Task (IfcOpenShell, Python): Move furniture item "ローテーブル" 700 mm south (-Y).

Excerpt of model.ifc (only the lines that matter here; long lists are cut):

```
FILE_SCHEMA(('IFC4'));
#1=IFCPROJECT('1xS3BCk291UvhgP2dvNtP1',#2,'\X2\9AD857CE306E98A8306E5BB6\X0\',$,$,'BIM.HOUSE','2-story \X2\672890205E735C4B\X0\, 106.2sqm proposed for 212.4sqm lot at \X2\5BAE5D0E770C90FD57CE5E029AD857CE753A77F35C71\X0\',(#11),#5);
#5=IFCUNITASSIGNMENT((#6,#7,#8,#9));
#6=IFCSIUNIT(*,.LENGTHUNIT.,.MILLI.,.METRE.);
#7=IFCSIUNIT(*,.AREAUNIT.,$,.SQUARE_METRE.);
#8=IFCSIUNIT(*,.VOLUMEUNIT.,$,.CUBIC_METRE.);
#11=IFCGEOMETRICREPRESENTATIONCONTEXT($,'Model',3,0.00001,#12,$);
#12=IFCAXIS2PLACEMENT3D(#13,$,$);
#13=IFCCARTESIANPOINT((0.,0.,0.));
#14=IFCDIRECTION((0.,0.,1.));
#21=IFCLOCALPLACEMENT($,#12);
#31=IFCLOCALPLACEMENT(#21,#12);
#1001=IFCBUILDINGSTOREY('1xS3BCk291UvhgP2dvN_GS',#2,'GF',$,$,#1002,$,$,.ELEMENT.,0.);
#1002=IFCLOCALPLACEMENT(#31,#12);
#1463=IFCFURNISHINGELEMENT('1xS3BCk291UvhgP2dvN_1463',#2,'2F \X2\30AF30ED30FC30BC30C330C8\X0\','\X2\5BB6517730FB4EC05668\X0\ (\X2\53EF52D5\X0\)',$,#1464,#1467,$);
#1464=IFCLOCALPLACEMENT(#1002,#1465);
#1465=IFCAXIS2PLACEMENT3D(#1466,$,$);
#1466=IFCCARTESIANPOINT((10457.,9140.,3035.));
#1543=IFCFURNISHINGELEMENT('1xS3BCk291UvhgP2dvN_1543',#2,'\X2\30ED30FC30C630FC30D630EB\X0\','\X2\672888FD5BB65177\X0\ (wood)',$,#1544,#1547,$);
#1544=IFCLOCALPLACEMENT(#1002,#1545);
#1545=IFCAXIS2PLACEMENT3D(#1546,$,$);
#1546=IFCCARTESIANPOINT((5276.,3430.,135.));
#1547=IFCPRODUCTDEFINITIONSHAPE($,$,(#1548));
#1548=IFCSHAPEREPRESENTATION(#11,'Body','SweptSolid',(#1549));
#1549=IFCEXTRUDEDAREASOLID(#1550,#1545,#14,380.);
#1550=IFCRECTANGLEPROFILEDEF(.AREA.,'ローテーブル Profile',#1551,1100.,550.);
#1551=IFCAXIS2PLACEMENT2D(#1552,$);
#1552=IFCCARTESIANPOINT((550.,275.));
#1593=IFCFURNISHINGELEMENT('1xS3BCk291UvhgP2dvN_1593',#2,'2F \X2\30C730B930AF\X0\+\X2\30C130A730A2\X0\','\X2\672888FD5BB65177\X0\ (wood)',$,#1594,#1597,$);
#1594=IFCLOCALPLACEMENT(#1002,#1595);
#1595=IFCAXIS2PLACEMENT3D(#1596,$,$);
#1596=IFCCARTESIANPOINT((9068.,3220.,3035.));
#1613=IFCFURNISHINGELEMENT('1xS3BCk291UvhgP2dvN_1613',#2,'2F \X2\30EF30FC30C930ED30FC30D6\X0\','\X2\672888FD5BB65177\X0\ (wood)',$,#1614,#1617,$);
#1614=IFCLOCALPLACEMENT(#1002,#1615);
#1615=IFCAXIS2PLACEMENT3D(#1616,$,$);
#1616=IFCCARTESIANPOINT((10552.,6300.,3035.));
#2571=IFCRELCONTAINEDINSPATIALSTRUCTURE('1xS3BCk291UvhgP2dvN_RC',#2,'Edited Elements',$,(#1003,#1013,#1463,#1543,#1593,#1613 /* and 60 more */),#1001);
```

```python
import ifcopenshell
import ifcopenshell.api.geometry
import ifcopenshell.util.placement
import ifcopenshell.util.unit

model = ifcopenshell.open("model.ifc")
unit_scale = ifcopenshell.util.unit.calculate_unit_scale(model)

item = model.by_guid("1xS3BCk291UvhgP2dvN_1543")
matrix = ifcopenshell.util.placement.get_local_placement(item.ObjectPlacement)
matrix[1, 3] -= 0.7 / unit_scale
ifcopenshell.api.geometry.edit_object_placement(model, product=item, matrix=matrix, is_si=False)

print(ifcopenshell.util.placement.get_local_placement(item.ObjectPlacement).round(3) + 0.0)

model.write("model_v2.ifc")
```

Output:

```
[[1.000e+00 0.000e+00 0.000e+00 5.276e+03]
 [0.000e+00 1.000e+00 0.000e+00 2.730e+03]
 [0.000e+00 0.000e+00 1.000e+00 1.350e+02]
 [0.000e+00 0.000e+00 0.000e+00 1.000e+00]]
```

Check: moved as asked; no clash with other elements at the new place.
